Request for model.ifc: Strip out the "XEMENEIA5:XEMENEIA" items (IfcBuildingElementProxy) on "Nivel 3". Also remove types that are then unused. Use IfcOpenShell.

First a look at what the model holds.

```python
import ifcopenshell
import ifcopenshell.util.element

model = ifcopenshell.open("model.ifc")
print(model.schema)
storey = next(s for s in model.by_type("IfcBuildingStorey") if s.Name == "Nivel 3")
proxies = [e for e in ifcopenshell.util.element.get_decomposition(storey) if e.is_a("IfcBuildingElementProxy")]
seen = {}
for e in proxies:
    element_type = ifcopenshell.util.element.get_type(e)
    name = element_type.Name if element_type not in (None, e) else None
    seen[name] = seen.get(name, 0) + 1
for name, count in sorted(seen.items(), key=str):
    print(count, "x", name)
```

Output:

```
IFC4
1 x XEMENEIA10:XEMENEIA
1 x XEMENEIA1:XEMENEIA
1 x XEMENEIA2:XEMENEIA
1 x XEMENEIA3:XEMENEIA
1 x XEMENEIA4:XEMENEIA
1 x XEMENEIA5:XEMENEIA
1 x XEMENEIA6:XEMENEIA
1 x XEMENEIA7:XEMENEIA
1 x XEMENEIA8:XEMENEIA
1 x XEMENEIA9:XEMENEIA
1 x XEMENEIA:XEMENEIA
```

```python
import ifcopenshell
import ifcopenshell.api.root
import ifcopenshell.util.element

model = ifcopenshell.open("model.ifc")

storey = next(s for s in model.by_type("IfcBuildingStorey") if s.Name == "Nivel 3")
proxies = [e for e in ifcopenshell.util.element.get_decomposition(storey) if e.is_a("IfcBuildingElementProxy")]
targets = [e for e in proxies if (t := ifcopenshell.util.element.get_type(e)) not in (None, e) and t.Name == "XEMENEIA5:XEMENEIA"]
types = {ifcopenshell.util.element.get_type(e) for e in targets} - {None, *targets}

for e in targets:
    ifcopenshell.api.root.remove_product(model, product=e)
print(len(targets), "removed")

unused = [t for t in types if not ifcopenshell.util.element.get_types(t)]
for t in unused:
    ifcopenshell.api.root.remove_product(model, product=t)
print(len(unused), "unused types removed")

model.write("model_rev.ifc")
```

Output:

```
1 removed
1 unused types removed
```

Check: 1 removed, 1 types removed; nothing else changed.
